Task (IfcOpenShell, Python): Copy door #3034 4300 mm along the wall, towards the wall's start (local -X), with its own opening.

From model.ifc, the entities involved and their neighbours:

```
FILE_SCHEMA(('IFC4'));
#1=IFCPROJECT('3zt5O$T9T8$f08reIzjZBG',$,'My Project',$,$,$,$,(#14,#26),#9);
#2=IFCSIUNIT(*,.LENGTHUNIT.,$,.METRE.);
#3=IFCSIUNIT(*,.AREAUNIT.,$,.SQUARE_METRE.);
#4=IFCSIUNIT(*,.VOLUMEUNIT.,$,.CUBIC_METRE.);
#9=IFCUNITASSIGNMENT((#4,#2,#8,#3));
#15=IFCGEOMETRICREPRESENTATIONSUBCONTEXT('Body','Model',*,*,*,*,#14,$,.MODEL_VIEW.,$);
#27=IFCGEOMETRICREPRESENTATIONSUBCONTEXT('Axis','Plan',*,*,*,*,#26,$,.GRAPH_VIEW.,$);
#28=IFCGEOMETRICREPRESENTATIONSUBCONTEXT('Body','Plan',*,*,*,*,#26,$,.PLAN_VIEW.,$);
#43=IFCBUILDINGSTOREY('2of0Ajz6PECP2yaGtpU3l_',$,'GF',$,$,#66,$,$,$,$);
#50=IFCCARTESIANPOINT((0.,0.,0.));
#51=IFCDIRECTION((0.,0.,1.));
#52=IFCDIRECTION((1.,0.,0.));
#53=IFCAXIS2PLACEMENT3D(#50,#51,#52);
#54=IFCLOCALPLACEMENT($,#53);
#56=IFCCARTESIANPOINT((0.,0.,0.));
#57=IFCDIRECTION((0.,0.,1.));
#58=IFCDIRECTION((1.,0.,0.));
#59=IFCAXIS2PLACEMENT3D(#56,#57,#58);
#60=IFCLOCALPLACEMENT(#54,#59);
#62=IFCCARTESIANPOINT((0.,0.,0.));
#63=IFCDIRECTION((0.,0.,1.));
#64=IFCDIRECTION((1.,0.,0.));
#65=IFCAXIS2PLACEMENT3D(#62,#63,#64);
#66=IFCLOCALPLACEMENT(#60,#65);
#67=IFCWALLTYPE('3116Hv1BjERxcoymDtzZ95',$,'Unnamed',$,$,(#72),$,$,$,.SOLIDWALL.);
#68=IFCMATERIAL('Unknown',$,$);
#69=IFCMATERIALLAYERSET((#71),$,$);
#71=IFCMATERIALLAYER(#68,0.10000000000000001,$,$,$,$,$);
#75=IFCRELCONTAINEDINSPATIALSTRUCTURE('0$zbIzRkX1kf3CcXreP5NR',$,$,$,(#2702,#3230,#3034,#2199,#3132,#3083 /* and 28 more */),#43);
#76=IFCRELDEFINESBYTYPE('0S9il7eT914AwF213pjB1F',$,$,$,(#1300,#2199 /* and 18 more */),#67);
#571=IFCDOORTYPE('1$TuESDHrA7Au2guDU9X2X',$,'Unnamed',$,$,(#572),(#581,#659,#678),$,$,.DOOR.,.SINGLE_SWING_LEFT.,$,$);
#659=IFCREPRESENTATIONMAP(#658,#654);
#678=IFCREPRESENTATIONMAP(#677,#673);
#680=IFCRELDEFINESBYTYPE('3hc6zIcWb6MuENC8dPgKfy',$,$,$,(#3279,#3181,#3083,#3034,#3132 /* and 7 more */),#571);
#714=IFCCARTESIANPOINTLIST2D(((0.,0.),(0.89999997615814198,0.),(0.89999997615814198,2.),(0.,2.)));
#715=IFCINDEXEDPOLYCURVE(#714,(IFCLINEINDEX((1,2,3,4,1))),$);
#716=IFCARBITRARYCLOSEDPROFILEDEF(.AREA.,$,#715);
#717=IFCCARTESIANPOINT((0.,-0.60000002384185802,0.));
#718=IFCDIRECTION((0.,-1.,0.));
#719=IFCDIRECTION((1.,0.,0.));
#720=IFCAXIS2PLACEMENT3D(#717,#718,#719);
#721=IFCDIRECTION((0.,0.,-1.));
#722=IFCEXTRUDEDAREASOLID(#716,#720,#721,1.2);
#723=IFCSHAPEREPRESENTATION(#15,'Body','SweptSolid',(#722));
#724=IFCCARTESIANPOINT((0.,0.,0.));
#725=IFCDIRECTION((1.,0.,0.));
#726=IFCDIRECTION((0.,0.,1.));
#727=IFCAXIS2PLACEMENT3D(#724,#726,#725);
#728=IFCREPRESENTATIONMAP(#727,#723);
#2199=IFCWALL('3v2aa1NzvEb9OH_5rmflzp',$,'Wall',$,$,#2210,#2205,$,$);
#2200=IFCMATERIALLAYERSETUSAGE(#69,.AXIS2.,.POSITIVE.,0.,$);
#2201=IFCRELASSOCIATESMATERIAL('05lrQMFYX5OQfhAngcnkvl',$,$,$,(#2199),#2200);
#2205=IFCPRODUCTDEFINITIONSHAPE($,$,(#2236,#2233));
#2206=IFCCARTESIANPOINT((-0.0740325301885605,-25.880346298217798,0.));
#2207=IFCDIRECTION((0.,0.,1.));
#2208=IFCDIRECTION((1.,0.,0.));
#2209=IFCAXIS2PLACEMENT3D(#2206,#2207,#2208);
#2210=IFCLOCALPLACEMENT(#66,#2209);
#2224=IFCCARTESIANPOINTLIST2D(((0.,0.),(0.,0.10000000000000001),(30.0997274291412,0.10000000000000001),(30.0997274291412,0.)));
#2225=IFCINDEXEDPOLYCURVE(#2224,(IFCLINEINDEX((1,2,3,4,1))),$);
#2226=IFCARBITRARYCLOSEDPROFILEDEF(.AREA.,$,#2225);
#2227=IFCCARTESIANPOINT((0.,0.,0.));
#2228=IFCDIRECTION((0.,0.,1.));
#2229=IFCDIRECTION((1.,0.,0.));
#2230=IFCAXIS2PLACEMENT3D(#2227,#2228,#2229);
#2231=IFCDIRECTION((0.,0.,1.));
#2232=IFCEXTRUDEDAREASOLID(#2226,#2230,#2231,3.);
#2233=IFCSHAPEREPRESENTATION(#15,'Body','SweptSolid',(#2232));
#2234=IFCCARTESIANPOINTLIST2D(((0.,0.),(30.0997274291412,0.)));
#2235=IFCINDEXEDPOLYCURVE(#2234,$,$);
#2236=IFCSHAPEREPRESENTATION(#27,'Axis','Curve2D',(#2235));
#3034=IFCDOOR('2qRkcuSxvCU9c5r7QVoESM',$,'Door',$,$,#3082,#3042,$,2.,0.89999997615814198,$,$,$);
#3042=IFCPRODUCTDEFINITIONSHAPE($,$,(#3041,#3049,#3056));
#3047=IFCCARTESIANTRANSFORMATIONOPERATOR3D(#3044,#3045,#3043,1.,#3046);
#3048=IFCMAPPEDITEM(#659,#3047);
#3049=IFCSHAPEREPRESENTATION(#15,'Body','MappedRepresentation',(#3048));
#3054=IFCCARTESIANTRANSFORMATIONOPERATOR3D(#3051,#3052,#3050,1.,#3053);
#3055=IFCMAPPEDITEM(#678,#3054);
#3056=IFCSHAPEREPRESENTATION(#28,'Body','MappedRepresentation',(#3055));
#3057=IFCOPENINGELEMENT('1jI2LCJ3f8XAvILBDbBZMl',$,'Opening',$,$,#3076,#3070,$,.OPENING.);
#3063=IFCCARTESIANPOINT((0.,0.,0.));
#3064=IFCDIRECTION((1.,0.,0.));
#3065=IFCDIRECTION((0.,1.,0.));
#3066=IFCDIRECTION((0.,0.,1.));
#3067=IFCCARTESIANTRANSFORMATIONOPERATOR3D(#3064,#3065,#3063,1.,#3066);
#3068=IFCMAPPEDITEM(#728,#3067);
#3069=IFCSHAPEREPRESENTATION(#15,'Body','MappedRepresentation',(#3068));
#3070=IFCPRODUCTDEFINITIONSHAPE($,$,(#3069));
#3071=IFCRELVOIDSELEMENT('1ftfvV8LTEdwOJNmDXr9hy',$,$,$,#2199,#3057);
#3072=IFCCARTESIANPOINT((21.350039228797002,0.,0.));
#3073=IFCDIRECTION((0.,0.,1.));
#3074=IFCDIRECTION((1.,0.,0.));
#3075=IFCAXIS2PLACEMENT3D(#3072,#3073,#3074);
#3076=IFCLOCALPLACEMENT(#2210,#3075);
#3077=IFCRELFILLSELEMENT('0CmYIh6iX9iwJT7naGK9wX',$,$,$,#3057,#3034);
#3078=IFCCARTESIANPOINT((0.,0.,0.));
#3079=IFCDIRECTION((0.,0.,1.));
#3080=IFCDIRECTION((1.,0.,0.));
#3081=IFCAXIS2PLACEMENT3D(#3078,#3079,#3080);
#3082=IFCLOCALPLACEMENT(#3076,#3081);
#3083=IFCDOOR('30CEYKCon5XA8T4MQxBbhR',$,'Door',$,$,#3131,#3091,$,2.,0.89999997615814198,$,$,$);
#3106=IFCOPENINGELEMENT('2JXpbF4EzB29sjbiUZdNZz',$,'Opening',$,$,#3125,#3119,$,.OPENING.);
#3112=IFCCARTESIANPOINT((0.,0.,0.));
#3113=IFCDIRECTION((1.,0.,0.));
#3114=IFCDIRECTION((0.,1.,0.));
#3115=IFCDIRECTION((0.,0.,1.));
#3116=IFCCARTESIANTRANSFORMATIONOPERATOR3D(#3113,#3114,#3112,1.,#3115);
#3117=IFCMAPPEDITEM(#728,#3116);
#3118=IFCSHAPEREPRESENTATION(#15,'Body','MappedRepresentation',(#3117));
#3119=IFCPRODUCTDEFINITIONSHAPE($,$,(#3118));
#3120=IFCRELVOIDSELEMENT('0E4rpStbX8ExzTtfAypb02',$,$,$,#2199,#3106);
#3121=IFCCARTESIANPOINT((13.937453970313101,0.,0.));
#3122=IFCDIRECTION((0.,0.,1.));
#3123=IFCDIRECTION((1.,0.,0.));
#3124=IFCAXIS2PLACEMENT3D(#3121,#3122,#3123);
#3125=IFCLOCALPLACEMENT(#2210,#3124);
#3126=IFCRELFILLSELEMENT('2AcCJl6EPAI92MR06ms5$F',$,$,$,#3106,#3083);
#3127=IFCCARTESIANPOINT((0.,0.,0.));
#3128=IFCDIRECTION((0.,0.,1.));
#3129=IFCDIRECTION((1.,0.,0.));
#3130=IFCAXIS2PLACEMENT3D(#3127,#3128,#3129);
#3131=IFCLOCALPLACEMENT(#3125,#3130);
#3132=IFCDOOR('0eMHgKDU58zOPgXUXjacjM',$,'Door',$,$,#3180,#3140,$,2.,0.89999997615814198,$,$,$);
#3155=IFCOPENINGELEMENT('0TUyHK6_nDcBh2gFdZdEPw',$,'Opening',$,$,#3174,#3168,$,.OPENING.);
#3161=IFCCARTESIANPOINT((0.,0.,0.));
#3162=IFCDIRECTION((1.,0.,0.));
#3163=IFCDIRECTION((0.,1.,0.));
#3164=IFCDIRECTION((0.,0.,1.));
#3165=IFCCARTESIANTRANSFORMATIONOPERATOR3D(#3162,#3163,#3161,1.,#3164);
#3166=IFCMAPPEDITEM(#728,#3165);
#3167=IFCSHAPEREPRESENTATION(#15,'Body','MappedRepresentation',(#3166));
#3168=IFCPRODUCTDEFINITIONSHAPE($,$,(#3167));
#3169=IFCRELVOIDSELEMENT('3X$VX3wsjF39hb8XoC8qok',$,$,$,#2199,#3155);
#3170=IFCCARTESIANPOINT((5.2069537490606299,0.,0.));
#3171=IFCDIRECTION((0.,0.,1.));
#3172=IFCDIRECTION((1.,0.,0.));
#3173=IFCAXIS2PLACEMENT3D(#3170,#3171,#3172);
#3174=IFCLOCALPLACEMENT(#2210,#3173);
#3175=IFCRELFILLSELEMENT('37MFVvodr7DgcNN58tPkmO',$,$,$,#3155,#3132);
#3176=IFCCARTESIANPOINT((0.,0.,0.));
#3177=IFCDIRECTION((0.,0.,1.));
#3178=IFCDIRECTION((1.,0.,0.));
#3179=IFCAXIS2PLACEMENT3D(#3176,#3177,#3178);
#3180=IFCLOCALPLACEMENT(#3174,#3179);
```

```python
import ifcopenshell
import ifcopenshell.api.feature
import ifcopenshell.api.geometry
import ifcopenshell.api.root
import ifcopenshell.geom
import ifcopenshell.util.element
import ifcopenshell.util.placement
import ifcopenshell.util.shape
import ifcopenshell.util.unit

model = ifcopenshell.open("model.ifc")
unit_scale = ifcopenshell.util.unit.calculate_unit_scale(model)
settings = ifcopenshell.geom.settings()


def volume(element):
    """Net volume in cubic metres, openings subtracted."""
    shape = ifcopenshell.geom.create_shape(settings, element)
    return ifcopenshell.util.shape.get_volume(shape.geometry)


door = model.by_guid("2qRkcuSxvCU9c5r7QVoESM")
opening = door.FillsVoids[0].RelatingOpeningElement
wall = opening.VoidsElements[0].RelatingBuildingElement
before = volume(wall)
shift = ifcopenshell.util.placement.get_local_placement(wall.ObjectPlacement)[:3, 0] * -4.3 / unit_scale

# copy_class copies the void relationship, type, container and properties, but no geometry.
new_opening = ifcopenshell.api.root.copy_class(model, product=opening)
new_opening.Representation = ifcopenshell.util.element.copy_deep(
    model, opening.Representation, exclude=["IfcGeometricRepresentationContext", "IfcRepresentationMap"]
)
new_door = ifcopenshell.api.root.copy_class(model, product=door)
new_door.Representation = ifcopenshell.util.element.copy_deep(
    model, door.Representation, exclude=["IfcGeometricRepresentationContext", "IfcRepresentationMap"]
)
ifcopenshell.api.feature.add_filling(model, opening=new_opening, element=new_door)

for old, new in ((opening, new_opening), (door, new_door)):
    matrix = ifcopenshell.util.placement.get_local_placement(old.ObjectPlacement)
    matrix[:3, 3] += shift
    ifcopenshell.api.geometry.edit_object_placement(model, product=new, matrix=matrix, is_si=False)

after = volume(wall)

print(f"wall volume {before:.3f} -> {after:.3f} m3")

model.write("model_edited.ifc")
```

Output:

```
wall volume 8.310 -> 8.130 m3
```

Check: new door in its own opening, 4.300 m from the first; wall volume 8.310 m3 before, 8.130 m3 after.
